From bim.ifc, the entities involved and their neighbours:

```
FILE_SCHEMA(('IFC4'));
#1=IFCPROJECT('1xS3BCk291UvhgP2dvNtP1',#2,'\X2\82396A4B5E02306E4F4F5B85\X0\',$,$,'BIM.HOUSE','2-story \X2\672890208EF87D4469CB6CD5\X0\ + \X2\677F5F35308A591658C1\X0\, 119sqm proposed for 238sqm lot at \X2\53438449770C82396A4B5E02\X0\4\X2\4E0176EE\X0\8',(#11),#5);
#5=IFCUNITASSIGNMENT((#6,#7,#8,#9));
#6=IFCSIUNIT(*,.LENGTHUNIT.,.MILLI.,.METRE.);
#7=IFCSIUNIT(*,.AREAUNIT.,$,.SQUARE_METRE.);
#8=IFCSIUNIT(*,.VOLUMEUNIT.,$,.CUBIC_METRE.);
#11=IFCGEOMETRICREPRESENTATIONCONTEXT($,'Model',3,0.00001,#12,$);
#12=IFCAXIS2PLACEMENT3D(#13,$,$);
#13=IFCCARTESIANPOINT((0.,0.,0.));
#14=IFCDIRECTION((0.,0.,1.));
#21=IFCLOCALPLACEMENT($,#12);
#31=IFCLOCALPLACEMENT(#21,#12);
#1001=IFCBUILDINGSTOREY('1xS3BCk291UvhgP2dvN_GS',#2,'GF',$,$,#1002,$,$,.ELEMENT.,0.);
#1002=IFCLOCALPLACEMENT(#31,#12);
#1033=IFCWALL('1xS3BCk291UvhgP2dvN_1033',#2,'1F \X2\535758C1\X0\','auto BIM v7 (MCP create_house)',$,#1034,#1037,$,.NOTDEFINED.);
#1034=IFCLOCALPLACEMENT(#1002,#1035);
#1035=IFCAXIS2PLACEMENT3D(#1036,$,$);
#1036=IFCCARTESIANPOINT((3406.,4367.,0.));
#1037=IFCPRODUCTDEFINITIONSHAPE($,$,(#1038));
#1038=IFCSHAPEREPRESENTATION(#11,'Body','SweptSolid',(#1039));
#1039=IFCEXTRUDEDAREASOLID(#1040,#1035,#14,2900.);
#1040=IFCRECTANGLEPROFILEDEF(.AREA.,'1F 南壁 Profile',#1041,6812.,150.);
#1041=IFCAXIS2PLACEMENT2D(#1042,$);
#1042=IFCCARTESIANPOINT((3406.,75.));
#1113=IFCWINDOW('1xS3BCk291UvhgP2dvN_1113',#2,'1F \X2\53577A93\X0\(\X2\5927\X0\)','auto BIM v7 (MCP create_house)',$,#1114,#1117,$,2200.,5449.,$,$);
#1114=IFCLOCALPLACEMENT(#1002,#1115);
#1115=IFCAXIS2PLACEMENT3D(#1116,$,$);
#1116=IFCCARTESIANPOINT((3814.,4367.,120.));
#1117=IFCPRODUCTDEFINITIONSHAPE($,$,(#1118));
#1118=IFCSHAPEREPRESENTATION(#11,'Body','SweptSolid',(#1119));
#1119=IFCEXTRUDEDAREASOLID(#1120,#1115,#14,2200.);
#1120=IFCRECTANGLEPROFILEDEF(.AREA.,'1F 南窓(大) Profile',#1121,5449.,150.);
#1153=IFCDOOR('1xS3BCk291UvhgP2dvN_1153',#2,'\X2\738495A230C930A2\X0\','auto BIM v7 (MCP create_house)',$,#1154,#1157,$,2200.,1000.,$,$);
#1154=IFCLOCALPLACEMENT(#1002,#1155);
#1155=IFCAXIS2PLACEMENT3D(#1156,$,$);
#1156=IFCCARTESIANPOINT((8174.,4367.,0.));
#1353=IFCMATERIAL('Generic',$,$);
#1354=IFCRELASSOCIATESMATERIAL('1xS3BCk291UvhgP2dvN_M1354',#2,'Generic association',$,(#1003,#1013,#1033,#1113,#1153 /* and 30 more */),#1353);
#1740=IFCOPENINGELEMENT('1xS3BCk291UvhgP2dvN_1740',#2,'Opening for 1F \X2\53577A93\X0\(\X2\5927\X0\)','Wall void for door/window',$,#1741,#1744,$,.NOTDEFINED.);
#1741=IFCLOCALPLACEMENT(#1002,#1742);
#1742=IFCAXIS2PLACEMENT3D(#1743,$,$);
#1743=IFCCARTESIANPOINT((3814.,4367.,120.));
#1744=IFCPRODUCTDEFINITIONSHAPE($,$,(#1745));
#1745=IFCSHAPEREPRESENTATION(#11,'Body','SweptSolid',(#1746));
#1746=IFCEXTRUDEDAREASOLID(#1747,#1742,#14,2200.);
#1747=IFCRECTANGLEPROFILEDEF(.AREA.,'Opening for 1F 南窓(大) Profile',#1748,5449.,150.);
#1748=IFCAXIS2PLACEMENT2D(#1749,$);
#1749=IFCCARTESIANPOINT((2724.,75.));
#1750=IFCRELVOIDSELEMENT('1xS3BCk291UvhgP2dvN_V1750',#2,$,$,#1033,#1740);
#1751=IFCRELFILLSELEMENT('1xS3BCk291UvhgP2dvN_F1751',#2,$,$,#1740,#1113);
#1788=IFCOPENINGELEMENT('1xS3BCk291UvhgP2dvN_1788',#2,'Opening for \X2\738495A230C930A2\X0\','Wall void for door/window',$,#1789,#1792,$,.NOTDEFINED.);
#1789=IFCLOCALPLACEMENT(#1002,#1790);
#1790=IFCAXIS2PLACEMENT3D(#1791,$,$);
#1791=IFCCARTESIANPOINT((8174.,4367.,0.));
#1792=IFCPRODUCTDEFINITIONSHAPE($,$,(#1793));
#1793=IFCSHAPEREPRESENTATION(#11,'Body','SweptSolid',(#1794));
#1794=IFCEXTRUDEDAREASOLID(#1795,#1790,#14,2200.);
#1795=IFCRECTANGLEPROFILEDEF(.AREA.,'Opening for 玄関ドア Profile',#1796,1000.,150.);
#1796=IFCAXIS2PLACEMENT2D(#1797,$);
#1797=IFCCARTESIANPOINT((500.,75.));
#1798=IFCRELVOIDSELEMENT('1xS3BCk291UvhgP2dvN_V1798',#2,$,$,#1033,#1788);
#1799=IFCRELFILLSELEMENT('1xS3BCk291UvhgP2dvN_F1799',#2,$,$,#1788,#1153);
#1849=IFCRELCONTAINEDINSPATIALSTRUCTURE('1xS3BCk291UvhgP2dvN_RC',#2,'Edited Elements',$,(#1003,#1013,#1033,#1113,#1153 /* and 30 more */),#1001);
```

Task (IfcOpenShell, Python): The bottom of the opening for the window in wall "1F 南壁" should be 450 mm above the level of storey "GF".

```python
import numpy as np
import ifcopenshell
import ifcopenshell.api.geometry
import ifcopenshell.geom
import ifcopenshell.util.element
import ifcopenshell.util.placement
import ifcopenshell.util.shape
import ifcopenshell.util.unit

model = ifcopenshell.open("bim.ifc")
unit_scale = ifcopenshell.util.unit.calculate_unit_scale(model)

window = model.by_guid("1xS3BCk291UvhgP2dvN_1113")
opening = window.FillsVoids[0].RelatingOpeningElement
storey = ifcopenshell.util.element.get_container(window, ifc_class="IfcBuildingStorey")
level = ifcopenshell.util.placement.get_local_placement(storey.ObjectPlacement)[2, 3]

# The opening's origin need not be at the sill, so measure its lowest point.
shape = ifcopenshell.geom.create_shape(ifcopenshell.geom.settings(), opening)
bottom = ifcopenshell.util.shape.get_shape_bottom_elevation(shape, shape.geometry) / unit_scale
dz = level + 0.45 / unit_scale - bottom

shift = np.array([0.0, 0.0, dz])
# The window is not placed relative to its opening, so move both.
for product in (opening, window):
    matrix = ifcopenshell.util.placement.get_local_placement(product.ObjectPlacement)
    matrix[:3, 3] += shift
    ifcopenshell.api.geometry.edit_object_placement(model, product=product, matrix=matrix, is_si=False)

print(f"moved by {dz * unit_scale:+.3f} m")

model.write("bim_edited.ifc")
```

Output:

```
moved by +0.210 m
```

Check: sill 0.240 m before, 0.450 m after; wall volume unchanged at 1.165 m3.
